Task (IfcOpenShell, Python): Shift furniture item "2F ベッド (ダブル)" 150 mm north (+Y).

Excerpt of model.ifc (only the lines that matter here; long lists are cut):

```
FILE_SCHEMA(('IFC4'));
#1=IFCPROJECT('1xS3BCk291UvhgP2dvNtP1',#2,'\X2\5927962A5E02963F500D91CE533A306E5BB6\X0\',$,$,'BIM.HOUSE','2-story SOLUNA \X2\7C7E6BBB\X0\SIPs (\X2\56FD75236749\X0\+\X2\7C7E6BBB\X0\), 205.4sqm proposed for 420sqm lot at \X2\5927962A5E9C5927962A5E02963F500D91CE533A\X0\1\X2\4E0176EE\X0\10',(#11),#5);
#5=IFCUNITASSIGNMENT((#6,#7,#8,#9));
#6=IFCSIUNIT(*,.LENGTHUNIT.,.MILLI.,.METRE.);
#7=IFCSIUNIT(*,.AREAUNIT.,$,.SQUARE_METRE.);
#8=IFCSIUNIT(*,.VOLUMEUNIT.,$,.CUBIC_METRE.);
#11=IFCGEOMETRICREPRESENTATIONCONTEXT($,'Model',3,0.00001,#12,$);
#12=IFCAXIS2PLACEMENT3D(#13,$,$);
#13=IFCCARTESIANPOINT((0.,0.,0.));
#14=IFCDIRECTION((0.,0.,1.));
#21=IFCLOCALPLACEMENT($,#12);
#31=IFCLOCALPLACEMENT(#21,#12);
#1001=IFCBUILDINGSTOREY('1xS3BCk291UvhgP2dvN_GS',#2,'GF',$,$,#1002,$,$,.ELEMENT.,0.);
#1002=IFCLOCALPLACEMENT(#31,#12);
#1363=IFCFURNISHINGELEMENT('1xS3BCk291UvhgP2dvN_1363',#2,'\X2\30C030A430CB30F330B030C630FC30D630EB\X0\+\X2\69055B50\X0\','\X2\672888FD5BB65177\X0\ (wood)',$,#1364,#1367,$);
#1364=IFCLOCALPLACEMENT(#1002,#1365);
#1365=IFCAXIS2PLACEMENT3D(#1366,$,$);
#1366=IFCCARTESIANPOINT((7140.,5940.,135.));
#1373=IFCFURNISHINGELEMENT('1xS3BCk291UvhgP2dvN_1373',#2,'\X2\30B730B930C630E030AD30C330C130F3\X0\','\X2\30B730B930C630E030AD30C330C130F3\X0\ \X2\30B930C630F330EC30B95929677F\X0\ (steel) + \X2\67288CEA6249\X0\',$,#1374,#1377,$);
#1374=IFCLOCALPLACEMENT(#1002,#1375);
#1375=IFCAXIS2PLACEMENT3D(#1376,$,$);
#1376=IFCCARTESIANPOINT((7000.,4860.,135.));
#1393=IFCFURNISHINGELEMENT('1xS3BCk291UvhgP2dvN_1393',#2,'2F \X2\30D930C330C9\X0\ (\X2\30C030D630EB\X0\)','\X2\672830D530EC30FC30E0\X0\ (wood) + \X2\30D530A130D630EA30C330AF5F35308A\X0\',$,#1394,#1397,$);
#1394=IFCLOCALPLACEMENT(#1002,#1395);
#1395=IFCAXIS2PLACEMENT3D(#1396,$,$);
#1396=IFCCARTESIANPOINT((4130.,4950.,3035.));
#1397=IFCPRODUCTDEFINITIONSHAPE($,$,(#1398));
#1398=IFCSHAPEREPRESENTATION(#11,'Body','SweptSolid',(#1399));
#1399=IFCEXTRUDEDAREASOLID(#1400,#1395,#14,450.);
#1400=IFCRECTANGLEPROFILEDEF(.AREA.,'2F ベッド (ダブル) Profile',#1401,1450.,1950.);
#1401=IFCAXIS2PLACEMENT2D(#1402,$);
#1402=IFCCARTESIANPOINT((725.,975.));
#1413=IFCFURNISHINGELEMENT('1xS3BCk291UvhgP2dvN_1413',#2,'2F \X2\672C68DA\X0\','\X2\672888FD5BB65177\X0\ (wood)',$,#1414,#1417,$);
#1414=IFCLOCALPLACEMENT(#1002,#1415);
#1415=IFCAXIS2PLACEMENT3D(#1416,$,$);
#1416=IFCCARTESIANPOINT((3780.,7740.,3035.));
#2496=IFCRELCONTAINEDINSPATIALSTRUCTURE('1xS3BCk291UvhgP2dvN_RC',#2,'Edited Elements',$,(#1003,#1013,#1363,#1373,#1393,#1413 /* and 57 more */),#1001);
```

```python
import ifcopenshell
import ifcopenshell.api.geometry
import ifcopenshell.util.placement

model = ifcopenshell.open("model.ifc")

item = model.by_guid("1xS3BCk291UvhgP2dvN_1393")
matrix = ifcopenshell.util.placement.get_local_placement(item.ObjectPlacement)
matrix[1, 3] += 150.0
ifcopenshell.api.geometry.edit_object_placement(model, product=item, matrix=matrix, is_si=False)

print(ifcopenshell.util.placement.get_local_placement(item.ObjectPlacement).round(3) + 0.0)

model.write("model_v2.ifc")
```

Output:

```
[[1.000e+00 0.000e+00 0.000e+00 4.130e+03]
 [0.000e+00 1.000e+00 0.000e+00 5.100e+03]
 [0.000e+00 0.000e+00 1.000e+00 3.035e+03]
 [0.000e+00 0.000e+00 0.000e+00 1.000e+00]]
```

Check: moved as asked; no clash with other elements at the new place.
